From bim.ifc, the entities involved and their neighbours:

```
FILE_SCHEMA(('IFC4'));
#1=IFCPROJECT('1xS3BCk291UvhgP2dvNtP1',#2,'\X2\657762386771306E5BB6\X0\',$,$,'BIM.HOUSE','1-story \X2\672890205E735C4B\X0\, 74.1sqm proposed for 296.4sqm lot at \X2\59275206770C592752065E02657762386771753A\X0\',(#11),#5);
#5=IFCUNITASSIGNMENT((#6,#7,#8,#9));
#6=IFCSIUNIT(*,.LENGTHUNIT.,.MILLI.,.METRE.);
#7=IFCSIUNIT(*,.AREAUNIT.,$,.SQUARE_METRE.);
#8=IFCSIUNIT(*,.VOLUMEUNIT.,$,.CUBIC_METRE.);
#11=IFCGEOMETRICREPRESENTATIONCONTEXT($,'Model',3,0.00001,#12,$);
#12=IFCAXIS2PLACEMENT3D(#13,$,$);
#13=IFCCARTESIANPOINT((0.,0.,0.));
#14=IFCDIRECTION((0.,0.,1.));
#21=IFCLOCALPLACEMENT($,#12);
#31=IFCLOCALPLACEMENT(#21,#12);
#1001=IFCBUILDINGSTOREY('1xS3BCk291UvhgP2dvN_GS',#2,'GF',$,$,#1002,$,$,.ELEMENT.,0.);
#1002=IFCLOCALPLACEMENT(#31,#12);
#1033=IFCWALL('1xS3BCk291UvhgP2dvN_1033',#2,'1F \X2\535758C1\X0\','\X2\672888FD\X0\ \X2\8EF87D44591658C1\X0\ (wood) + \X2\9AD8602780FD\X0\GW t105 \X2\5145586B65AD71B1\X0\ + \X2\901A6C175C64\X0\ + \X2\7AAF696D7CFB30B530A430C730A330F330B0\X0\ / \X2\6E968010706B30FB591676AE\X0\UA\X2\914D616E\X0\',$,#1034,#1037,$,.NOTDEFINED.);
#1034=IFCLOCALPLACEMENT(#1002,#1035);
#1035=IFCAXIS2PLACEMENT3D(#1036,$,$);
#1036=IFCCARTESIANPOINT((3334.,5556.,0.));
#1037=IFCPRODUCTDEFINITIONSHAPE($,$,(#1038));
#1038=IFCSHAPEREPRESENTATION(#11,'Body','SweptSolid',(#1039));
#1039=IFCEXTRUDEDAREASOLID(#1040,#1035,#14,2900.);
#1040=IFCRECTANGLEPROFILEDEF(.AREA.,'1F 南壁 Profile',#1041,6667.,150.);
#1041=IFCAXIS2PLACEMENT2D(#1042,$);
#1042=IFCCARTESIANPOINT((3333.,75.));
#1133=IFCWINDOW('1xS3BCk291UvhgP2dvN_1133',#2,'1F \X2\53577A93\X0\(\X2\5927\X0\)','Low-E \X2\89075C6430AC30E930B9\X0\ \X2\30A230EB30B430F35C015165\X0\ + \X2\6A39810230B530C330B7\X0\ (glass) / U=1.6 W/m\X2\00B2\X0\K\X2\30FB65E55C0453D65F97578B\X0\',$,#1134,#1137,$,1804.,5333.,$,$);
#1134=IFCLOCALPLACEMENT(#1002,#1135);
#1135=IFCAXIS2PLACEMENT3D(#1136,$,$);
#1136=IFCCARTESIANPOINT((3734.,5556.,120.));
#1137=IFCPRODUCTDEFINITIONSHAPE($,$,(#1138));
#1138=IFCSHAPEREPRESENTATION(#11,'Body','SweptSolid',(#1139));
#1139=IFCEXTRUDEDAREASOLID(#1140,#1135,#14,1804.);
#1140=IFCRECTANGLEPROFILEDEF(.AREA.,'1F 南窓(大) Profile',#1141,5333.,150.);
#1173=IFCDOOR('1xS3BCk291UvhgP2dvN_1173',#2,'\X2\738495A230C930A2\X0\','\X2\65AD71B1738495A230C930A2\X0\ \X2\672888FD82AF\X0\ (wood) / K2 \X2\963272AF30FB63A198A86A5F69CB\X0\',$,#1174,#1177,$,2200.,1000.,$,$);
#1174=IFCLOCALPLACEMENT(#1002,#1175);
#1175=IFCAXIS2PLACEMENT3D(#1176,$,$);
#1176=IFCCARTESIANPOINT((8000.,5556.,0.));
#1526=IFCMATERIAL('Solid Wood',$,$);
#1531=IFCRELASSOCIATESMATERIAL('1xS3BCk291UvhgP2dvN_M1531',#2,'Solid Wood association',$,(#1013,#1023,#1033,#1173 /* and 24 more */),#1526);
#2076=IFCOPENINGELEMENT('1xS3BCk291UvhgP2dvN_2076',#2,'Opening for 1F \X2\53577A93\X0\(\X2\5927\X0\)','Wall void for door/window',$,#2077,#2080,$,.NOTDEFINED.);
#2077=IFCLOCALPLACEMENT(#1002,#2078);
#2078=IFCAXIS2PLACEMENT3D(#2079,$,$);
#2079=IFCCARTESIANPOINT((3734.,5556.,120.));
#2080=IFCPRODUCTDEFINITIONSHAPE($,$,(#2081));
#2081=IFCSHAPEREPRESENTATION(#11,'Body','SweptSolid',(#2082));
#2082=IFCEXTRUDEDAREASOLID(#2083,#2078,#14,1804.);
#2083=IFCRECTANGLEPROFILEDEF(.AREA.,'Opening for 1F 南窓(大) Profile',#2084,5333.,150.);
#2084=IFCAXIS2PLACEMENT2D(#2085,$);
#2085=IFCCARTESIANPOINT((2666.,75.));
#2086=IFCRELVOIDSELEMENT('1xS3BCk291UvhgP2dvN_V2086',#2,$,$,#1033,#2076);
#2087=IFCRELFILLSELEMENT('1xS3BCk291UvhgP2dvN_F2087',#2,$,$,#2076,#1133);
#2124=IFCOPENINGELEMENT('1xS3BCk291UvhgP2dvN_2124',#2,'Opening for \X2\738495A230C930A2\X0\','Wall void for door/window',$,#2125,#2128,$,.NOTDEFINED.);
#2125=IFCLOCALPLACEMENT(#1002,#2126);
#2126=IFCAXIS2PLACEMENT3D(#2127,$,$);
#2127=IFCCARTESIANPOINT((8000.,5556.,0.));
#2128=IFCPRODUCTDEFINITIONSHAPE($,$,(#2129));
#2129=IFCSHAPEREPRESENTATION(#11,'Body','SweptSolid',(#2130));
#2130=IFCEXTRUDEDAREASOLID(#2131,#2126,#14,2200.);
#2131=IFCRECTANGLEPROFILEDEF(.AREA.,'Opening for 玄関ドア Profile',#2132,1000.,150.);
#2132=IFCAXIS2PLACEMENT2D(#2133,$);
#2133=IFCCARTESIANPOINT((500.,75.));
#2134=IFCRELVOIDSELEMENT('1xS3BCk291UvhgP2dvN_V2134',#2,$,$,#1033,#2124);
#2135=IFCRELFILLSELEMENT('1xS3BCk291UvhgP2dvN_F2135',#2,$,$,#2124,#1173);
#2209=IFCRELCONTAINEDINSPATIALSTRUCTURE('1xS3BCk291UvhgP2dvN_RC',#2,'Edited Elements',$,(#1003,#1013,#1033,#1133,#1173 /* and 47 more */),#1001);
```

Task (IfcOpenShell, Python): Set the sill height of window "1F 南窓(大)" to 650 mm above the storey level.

```python
import numpy as np
import ifcopenshell
import ifcopenshell.api.geometry
import ifcopenshell.geom
import ifcopenshell.util.element
import ifcopenshell.util.placement
import ifcopenshell.util.shape
import ifcopenshell.util.unit

model = ifcopenshell.open("bim.ifc")
unit_scale = ifcopenshell.util.unit.calculate_unit_scale(model)

window = model.by_guid("1xS3BCk291UvhgP2dvN_1133")
opening = window.FillsVoids[0].RelatingOpeningElement
storey = ifcopenshell.util.element.get_container(window, ifc_class="IfcBuildingStorey")
level = ifcopenshell.util.placement.get_local_placement(storey.ObjectPlacement)[2, 3]

# The opening's origin need not be at the sill, so measure its lowest point.
shape = ifcopenshell.geom.create_shape(ifcopenshell.geom.settings(), opening)
bottom = ifcopenshell.util.shape.get_shape_bottom_elevation(shape, shape.geometry) / unit_scale
dz = level + 0.65 / unit_scale - bottom

shift = np.array([0.0, 0.0, dz])
# The window is not placed relative to its opening, so move both.
for product in (opening, window):
    matrix = ifcopenshell.util.placement.get_local_placement(product.ObjectPlacement)
    matrix[:3, 3] += shift
    ifcopenshell.api.geometry.edit_object_placement(model, product=product, matrix=matrix, is_si=False)

print(f"moved by {dz * unit_scale:+.3f} m")

model.write("bim_updated.ifc")
```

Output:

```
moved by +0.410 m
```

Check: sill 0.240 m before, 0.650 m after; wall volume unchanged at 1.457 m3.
